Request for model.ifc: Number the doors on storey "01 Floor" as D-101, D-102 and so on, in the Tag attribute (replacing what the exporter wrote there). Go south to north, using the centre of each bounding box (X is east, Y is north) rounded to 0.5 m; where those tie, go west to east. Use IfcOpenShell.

First a look at what the model holds.

```python
import ifcopenshell
import ifcopenshell.util.element
import ifcopenshell.util.placement

model = ifcopenshell.open("model.ifc")
print(model.schema)
storey = next(s for s in model.by_type("IfcBuildingStorey") if s.Name == "01 Floor")
doors = [e for e in ifcopenshell.util.element.get_decomposition(storey) if e.is_a("IfcDoor")]
for e in sorted(doors, key=lambda e: e.id()):
    origin = ifcopenshell.util.placement.get_local_placement(e.ObjectPlacement)[:3, 3]
    print(e.id(), e.Tag, e.Name, origin.round(2) + 0.0, sep=" | ")
```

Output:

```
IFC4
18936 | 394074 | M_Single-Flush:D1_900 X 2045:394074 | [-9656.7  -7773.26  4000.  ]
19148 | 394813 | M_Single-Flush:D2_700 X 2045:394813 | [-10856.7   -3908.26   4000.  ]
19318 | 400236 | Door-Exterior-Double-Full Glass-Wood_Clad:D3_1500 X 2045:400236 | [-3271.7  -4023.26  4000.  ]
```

```python
import ifcopenshell
import ifcopenshell.geom
import ifcopenshell.util.element
import ifcopenshell.util.shape

model = ifcopenshell.open("model.ifc")
settings = ifcopenshell.geom.settings()
settings.set("use-world-coords", True)


def centre(element):
    shape = ifcopenshell.geom.create_shape(settings, element)
    return ifcopenshell.util.shape.get_bbox_centroid(shape.geometry)


storey = next(s for s in model.by_type("IfcBuildingStorey") if s.Name == "01 Floor")
doors = [e for e in ifcopenshell.util.element.get_decomposition(storey) if e.is_a("IfcDoor")]

# Insertion points can sit at a corner or the storey origin, so sort by the geometry (in metres).
centres = {e: centre(e) for e in doors}
doors.sort(key=lambda e: (round(centres[e][1] / 0.5), centres[e][0]))

for i, e in enumerate(doors, start=1):
    number = f"D-1{i:02d}"
    e.Tag = number
    print(e.id(), number)

model.write("model_rev.ifc")
```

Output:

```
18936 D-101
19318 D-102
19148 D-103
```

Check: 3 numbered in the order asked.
